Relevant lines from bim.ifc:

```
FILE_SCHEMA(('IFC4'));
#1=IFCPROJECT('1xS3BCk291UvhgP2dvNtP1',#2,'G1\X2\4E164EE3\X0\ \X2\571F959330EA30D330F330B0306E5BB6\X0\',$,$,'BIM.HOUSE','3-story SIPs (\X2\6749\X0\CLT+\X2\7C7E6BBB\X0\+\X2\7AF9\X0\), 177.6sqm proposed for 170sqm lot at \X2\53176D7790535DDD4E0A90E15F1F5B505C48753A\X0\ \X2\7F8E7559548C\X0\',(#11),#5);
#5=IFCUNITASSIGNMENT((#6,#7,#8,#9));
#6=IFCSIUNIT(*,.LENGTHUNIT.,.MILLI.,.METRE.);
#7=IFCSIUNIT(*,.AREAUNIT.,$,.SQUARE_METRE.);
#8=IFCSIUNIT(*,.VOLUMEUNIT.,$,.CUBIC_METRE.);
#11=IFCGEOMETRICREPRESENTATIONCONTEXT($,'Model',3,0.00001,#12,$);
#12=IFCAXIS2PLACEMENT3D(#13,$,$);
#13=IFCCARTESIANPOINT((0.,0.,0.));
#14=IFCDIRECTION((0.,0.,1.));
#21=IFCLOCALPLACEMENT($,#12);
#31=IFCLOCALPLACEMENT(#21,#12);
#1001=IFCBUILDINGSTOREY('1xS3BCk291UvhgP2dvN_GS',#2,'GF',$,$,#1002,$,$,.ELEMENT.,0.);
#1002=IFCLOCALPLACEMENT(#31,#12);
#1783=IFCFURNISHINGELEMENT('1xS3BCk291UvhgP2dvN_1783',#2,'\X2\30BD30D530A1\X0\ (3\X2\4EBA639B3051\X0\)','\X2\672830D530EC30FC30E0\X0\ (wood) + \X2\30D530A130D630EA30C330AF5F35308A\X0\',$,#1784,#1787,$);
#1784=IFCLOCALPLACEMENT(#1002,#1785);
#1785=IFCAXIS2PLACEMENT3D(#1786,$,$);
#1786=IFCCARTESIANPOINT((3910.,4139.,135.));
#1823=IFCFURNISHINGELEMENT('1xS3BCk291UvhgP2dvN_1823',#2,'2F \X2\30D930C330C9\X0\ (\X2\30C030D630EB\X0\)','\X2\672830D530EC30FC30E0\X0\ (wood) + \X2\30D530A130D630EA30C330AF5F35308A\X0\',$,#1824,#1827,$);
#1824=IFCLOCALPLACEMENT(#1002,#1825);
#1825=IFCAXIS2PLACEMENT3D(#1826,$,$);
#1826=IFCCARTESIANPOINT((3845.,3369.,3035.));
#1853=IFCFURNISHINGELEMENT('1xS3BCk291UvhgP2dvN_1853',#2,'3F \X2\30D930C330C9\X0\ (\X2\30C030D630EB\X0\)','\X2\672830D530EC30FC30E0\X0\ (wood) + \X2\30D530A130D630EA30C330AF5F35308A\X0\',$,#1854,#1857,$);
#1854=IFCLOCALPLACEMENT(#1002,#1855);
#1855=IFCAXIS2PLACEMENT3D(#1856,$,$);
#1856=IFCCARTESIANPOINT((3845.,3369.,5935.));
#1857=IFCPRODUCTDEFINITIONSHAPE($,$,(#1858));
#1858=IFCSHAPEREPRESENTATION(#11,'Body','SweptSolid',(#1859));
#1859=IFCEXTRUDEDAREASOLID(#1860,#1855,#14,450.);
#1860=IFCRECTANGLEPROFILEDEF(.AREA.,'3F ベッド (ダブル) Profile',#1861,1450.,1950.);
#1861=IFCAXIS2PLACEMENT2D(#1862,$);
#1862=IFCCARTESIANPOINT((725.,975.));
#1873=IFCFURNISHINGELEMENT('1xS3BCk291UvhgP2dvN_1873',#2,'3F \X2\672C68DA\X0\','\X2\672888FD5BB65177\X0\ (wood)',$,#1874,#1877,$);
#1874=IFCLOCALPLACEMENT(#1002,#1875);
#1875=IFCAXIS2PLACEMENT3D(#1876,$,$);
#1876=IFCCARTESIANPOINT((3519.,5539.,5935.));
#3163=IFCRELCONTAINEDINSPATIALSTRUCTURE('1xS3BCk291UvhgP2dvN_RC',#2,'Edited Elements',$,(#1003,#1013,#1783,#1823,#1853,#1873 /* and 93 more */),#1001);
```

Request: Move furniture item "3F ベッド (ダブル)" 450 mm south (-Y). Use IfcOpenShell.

```python
import ifcopenshell
import ifcopenshell.api.geometry
import ifcopenshell.util.placement
import ifcopenshell.util.unit

model = ifcopenshell.open("bim.ifc")
unit_scale = ifcopenshell.util.unit.calculate_unit_scale(model)

item = model.by_guid("1xS3BCk291UvhgP2dvN_1853")
matrix = ifcopenshell.util.placement.get_local_placement(item.ObjectPlacement)
matrix[1, 3] -= 0.45 / unit_scale
ifcopenshell.api.geometry.edit_object_placement(model, product=item, matrix=matrix, is_si=False)

print(ifcopenshell.util.placement.get_local_placement(item.ObjectPlacement).round(3) + 0.0)

model.write("bim-out.ifc")
```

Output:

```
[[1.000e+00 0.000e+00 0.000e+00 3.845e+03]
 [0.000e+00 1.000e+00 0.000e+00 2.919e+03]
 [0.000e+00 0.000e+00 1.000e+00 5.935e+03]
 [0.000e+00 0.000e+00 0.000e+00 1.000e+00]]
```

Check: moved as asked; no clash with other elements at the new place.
